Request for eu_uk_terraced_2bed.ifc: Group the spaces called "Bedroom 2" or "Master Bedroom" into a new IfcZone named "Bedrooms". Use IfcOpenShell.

First a look at what the model holds.

```python
import ifcopenshell

model = ifcopenshell.open("eu_uk_terraced_2bed.ifc")
print(model.schema)
seen = {}
for space in model.by_type("IfcSpace"):
    seen[space.LongName] = seen.get(space.LongName, 0) + 1
for name, count in sorted(seen.items(), key=str):
    print(count, "x", name)
print("zones:", [z.Name for z in model.by_type("IfcZone")][:20])
```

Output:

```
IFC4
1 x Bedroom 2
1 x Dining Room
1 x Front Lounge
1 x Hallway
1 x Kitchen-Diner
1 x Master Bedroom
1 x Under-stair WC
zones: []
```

```python
import ifcopenshell
import ifcopenshell.api.group
import ifcopenshell.api.root

model = ifcopenshell.open("eu_uk_terraced_2bed.ifc")

names = {"Bedroom 2", "Master Bedroom"}
spaces = [s for s in model.by_type("IfcSpace") if s.LongName in names]

zone = ifcopenshell.api.root.create_entity(model, ifc_class="IfcZone", name="Bedrooms")
ifcopenshell.api.group.assign_group(model, products=spaces, group=zone)
print(len(spaces), "spaces in", zone.Name)

model.write("eu_uk_terraced_2bed_updated.ifc")
```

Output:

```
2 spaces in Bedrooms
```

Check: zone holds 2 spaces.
